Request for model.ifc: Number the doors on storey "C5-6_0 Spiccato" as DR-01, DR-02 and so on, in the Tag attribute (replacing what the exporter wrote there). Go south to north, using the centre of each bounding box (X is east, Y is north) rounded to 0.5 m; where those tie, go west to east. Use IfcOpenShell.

First a look at what the model holds.

```python
import ifcopenshell
import ifcopenshell.util.element
import ifcopenshell.util.placement

model = ifcopenshell.open("model.ifc")
print(model.schema)
storey = next(s for s in model.by_type("IfcBuildingStorey") if s.Name == "C5-6_0 Spiccato")
doors = [e for e in ifcopenshell.util.element.get_decomposition(storey) if e.is_a("IfcDoor")]
for e in sorted(doors, key=lambda e: e.id()):
    origin = ifcopenshell.util.placement.get_local_placement(e.ObjectPlacement)[:3, 3]
    print(e.id(), e.Tag, e.Name, origin.round(2) + 0.0, sep=" | ")
```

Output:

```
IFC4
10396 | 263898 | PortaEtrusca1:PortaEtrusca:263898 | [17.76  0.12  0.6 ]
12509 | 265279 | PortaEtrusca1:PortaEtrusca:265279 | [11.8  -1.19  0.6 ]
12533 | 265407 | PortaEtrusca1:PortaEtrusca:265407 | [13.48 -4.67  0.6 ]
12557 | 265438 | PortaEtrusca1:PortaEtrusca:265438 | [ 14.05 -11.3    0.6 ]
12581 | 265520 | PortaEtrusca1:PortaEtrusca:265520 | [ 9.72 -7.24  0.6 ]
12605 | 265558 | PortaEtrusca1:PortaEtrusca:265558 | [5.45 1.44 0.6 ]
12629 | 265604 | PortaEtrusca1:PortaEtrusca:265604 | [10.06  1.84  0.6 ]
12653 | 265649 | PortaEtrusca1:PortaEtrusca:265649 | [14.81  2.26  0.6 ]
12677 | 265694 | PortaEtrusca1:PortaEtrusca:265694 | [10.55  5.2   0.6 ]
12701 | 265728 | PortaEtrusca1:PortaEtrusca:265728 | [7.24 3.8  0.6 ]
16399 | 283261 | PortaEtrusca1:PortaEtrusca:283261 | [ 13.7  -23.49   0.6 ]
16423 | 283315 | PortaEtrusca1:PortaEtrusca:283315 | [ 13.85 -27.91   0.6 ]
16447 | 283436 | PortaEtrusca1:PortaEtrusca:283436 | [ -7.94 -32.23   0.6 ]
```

```python
import ifcopenshell
import ifcopenshell.geom
import ifcopenshell.util.element
import ifcopenshell.util.shape

model = ifcopenshell.open("model.ifc")
settings = ifcopenshell.geom.settings()
settings.set("use-world-coords", True)


def centre(element):
    shape = ifcopenshell.geom.create_shape(settings, element)
    return ifcopenshell.util.shape.get_bbox_centroid(shape.geometry)


storey = next(s for s in model.by_type("IfcBuildingStorey") if s.Name == "C5-6_0 Spiccato")
doors = [e for e in ifcopenshell.util.element.get_decomposition(storey) if e.is_a("IfcDoor")]

# Insertion points can sit at a corner or the storey origin, so sort by the geometry (in metres).
centres = {e: centre(e) for e in doors}
doors.sort(key=lambda e: (round(centres[e][1] / 0.5), centres[e][0]))

for i, e in enumerate(doors, start=1):
    number = f"DR-{i:02d}"
    e.Tag = number
    print(e.id(), number)

model.write("model_rev.ifc")
```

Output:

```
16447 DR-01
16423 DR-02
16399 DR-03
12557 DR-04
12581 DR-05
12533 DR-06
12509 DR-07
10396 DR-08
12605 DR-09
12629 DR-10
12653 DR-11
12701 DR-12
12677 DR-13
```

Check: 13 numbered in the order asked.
